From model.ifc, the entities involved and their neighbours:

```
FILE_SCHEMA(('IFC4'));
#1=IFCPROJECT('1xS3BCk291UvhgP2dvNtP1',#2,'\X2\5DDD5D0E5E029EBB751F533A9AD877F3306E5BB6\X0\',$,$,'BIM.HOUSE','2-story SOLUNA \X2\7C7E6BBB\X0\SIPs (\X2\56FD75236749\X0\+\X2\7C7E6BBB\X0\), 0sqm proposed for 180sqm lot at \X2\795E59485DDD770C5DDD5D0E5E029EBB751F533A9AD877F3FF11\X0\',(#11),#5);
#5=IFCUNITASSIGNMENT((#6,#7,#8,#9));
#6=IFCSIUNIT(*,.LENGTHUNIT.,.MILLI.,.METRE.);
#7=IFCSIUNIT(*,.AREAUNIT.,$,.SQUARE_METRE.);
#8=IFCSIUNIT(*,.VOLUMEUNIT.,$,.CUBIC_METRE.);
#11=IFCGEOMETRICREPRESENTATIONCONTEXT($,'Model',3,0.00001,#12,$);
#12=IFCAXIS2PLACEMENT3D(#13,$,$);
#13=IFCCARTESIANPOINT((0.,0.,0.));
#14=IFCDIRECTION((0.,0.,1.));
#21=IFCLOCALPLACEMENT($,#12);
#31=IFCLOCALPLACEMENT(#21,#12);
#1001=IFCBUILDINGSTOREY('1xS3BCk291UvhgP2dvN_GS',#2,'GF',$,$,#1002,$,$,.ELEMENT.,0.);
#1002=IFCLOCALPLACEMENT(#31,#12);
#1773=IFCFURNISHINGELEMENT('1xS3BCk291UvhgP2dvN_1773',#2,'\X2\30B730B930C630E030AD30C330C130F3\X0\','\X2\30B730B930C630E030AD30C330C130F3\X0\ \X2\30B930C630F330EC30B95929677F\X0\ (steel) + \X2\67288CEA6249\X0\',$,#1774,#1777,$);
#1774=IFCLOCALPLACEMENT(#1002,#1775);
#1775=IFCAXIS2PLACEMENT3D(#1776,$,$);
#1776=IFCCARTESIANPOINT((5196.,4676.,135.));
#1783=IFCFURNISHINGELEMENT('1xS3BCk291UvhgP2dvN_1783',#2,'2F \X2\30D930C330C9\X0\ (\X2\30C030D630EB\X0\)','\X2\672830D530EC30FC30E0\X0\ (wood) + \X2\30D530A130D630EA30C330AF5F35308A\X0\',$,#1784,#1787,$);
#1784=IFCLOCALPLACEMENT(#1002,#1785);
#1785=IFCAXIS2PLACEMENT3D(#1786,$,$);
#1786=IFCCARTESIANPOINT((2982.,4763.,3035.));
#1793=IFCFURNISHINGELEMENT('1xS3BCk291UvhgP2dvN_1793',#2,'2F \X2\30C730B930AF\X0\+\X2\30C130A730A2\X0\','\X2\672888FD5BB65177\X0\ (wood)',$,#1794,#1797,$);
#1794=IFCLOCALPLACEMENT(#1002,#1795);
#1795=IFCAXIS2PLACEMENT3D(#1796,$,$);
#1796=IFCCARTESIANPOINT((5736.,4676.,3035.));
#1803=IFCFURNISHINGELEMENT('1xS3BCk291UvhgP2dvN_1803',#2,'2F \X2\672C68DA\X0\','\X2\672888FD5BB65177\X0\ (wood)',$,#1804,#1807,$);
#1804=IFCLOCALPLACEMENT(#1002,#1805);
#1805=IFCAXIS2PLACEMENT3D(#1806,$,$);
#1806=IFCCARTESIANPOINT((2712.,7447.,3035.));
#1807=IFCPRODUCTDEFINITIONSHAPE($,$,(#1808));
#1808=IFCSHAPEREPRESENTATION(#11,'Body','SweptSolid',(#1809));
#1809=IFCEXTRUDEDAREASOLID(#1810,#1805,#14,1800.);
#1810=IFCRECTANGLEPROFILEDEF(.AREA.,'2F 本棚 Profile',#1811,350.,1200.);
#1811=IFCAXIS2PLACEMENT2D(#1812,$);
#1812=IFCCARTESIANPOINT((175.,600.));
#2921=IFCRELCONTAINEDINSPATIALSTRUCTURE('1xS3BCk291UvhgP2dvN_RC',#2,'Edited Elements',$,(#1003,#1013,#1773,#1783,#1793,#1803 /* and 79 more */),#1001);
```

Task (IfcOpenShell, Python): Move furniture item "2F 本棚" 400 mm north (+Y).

```python
import ifcopenshell
import ifcopenshell.api.geometry
import ifcopenshell.util.placement
import ifcopenshell.util.unit

model = ifcopenshell.open("model.ifc")
unit_scale = ifcopenshell.util.unit.calculate_unit_scale(model)

item = model.by_guid("1xS3BCk291UvhgP2dvN_1803")
matrix = ifcopenshell.util.placement.get_local_placement(item.ObjectPlacement)
matrix[1, 3] += 0.4 / unit_scale
ifcopenshell.api.geometry.edit_object_placement(model, product=item, matrix=matrix, is_si=False)

print(ifcopenshell.util.placement.get_local_placement(item.ObjectPlacement).round(3) + 0.0)

model.write("model_updated.ifc")
```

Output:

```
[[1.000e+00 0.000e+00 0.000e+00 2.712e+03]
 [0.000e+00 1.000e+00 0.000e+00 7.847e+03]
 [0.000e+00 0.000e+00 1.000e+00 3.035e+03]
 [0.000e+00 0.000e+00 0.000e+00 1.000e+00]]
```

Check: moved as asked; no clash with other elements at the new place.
